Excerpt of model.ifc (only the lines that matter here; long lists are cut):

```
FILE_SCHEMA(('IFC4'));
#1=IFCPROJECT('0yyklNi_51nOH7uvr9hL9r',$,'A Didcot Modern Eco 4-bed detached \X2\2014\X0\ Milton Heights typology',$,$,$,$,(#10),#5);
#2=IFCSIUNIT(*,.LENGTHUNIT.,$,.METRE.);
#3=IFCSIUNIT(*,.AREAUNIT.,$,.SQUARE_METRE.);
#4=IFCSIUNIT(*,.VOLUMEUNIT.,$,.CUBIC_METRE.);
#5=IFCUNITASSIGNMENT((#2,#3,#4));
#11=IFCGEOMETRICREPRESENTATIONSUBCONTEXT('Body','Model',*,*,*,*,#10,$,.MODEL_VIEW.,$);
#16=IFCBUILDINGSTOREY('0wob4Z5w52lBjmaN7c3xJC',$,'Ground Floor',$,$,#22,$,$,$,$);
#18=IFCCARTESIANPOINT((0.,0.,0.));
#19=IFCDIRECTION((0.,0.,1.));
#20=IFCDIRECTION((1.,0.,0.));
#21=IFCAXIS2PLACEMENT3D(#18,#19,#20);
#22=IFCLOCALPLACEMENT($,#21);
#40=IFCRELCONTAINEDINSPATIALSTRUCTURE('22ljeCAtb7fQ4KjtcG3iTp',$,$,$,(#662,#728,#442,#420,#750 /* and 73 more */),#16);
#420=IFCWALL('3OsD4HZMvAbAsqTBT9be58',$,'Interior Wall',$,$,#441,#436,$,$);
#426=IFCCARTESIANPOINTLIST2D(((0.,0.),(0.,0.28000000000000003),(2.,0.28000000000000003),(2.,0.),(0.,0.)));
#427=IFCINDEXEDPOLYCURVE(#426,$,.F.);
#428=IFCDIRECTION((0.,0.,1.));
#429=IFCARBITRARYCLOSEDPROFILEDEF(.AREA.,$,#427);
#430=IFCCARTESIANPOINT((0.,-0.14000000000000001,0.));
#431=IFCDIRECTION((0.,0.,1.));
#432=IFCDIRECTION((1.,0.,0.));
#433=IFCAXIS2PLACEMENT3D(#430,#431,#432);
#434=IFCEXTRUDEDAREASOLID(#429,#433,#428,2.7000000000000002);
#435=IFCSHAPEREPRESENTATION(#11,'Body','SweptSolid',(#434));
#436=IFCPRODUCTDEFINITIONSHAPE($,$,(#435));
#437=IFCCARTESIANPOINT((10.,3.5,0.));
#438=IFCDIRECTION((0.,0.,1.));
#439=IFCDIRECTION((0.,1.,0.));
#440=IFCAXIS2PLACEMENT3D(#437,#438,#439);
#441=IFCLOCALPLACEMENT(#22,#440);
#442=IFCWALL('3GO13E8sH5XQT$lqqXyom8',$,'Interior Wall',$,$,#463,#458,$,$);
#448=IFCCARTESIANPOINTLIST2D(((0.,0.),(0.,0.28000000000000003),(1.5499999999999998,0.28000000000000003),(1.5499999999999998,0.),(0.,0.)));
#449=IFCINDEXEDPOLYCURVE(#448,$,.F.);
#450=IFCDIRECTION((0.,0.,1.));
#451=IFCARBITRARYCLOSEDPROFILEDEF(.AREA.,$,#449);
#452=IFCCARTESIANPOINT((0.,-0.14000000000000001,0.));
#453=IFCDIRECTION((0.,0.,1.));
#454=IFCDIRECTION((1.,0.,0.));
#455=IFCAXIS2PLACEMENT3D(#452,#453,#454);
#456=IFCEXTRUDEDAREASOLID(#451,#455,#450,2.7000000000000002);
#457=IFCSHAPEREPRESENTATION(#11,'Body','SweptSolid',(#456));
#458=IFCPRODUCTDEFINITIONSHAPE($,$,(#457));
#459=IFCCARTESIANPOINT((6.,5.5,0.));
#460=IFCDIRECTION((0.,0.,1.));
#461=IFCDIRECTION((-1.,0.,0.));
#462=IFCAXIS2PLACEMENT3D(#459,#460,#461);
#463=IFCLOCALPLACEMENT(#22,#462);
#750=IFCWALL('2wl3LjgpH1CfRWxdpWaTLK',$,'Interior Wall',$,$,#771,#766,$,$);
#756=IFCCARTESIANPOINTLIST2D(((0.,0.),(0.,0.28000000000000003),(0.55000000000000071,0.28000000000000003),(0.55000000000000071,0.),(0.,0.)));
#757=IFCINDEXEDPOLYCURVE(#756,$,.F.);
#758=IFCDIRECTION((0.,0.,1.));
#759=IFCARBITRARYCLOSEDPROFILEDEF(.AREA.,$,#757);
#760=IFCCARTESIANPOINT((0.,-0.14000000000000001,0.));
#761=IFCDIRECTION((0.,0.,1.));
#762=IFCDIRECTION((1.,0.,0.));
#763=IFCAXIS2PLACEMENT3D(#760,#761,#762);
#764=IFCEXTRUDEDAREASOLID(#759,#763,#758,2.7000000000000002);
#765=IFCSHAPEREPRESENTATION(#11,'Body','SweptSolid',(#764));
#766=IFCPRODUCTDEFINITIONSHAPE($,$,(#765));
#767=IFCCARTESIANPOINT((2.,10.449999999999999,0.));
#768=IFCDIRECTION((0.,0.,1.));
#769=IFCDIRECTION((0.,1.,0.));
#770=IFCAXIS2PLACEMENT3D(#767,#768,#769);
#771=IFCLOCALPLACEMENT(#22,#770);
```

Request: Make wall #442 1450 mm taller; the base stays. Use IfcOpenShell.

```python
import ifcopenshell
import ifcopenshell.geom
import ifcopenshell.util.representation
import ifcopenshell.util.shape

model = ifcopenshell.open("model.ifc")
settings = ifcopenshell.geom.settings()


def volume(element):
    """Net volume in cubic metres, openings subtracted."""
    shape = ifcopenshell.geom.create_shape(settings, element)
    return ifcopenshell.util.shape.get_volume(shape.geometry)


wall = model.by_id(442)
before = volume(wall)

body = ifcopenshell.util.representation.get_representation(wall, "Model", "Body")
solid = body.Items[0]
old_height = solid.Depth
solid.Depth += 1.45
after = volume(wall)

print(f"height {old_height:g} -> {solid.Depth:g}, volume {before:.3f} -> {after:.3f} m3")

model.write("model-out.ifc")
```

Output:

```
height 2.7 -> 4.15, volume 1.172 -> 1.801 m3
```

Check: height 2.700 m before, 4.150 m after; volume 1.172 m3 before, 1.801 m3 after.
